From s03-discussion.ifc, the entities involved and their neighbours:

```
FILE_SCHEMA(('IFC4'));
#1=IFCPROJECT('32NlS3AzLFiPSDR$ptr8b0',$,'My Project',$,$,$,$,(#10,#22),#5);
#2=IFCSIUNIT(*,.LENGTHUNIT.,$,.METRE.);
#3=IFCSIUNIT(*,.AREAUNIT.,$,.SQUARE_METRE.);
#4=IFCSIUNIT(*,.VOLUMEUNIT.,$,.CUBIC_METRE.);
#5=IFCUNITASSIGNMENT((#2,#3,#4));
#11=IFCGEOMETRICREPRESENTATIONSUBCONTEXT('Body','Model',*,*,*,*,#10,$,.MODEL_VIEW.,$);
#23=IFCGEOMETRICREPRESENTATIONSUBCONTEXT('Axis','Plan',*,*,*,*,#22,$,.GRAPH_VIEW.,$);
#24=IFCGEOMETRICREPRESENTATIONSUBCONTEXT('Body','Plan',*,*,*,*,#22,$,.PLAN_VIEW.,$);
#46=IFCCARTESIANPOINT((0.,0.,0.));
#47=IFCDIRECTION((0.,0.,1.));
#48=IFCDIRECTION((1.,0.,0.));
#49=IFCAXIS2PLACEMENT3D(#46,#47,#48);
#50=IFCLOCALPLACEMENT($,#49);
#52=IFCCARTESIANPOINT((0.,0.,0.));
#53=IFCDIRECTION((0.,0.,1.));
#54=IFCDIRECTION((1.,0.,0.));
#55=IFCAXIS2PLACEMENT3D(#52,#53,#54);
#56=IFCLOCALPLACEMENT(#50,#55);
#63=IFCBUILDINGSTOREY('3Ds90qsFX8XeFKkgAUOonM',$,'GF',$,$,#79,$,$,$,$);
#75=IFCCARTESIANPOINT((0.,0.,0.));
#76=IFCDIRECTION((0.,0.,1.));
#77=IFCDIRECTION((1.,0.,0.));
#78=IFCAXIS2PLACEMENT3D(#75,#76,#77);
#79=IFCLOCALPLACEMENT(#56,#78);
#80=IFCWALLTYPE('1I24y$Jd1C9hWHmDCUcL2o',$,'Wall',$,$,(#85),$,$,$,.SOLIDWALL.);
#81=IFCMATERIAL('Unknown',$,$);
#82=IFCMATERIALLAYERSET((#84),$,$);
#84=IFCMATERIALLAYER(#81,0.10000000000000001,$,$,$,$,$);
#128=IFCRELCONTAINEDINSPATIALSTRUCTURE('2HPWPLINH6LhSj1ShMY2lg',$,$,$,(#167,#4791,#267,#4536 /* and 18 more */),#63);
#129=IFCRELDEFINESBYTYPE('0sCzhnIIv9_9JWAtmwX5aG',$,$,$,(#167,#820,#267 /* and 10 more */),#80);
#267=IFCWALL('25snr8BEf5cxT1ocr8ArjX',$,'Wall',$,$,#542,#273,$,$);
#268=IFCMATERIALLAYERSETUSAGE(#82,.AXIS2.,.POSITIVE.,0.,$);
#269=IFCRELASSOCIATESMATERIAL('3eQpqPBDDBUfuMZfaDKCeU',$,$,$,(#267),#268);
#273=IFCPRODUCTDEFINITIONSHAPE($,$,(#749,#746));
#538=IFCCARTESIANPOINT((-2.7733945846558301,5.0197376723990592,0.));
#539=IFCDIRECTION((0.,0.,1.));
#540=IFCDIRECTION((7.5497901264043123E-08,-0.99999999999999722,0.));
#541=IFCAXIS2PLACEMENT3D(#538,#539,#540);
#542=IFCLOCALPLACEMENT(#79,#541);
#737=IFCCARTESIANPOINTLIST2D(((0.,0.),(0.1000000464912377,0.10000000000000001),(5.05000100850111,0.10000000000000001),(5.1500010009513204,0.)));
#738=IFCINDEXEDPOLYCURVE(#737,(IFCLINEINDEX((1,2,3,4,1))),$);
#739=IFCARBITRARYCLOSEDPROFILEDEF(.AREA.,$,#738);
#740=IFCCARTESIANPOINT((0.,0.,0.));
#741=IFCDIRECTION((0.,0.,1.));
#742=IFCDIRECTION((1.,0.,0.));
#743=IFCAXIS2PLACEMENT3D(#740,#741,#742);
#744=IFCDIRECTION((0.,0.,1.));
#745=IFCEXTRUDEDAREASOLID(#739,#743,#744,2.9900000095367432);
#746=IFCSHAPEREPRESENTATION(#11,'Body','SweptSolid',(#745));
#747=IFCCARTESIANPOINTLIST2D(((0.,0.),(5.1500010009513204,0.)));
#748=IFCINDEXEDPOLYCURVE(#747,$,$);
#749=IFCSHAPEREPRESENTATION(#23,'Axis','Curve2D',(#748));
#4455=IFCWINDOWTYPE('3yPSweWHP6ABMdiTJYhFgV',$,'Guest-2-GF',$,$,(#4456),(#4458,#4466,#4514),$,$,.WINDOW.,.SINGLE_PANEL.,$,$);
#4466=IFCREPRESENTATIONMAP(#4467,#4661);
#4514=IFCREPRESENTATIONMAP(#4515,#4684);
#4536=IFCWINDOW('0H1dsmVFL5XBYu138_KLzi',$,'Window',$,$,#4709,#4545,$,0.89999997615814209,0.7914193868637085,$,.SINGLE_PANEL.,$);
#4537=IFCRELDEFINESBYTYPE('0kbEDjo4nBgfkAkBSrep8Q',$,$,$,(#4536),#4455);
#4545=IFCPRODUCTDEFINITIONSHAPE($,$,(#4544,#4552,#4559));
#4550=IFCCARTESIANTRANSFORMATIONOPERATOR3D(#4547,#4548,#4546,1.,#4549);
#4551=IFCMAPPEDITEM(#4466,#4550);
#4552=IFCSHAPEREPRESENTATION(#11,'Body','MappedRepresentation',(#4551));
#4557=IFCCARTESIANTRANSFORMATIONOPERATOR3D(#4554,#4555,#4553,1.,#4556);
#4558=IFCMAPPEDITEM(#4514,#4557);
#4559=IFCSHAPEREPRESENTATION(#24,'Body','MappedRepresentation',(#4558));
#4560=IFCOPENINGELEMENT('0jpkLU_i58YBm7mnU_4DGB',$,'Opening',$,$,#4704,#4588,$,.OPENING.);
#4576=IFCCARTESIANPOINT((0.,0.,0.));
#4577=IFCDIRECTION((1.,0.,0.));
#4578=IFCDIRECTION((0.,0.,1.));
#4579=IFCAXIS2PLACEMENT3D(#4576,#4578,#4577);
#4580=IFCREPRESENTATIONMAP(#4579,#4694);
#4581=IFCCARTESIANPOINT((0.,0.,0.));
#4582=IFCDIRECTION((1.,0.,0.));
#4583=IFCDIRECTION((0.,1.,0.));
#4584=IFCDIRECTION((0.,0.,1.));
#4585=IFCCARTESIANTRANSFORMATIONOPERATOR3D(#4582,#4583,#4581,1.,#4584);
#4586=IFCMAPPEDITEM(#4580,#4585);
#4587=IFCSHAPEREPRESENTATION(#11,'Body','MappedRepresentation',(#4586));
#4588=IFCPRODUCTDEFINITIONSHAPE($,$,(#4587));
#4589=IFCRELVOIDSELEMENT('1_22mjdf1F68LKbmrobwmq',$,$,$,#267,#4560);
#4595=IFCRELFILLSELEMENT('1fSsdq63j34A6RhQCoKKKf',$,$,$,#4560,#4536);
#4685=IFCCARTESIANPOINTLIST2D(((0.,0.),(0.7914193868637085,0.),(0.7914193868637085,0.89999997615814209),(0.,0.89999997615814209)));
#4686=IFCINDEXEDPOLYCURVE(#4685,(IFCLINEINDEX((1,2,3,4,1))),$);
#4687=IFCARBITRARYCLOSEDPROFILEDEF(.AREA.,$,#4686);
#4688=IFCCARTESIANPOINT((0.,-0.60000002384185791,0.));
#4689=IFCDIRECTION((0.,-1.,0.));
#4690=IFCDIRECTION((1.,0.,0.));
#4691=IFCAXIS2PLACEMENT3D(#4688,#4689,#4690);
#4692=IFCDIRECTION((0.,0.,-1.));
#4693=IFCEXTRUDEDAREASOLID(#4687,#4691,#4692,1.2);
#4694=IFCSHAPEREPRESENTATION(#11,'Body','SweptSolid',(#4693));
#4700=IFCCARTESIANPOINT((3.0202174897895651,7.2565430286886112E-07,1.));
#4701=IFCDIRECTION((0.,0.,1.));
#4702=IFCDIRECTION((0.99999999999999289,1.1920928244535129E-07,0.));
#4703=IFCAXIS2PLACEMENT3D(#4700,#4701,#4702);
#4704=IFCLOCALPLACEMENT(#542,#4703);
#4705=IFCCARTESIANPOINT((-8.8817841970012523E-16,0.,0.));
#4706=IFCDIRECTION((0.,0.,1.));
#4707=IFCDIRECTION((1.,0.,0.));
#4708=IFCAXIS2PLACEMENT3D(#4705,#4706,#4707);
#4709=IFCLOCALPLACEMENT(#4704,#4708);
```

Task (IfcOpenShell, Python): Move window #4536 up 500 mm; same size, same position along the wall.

```python
import numpy as np
import ifcopenshell
import ifcopenshell.api.geometry
import ifcopenshell.util.placement
import ifcopenshell.util.unit

model = ifcopenshell.open("s03-discussion.ifc")
unit_scale = ifcopenshell.util.unit.calculate_unit_scale(model)

window = model.by_guid("0H1dsmVFL5XBYu138_KLzi")
opening = window.FillsVoids[0].RelatingOpeningElement
dz = 0.5 / unit_scale

shift = np.array([0.0, 0.0, dz])
# The window is placed relative to its opening, so it follows when the opening moves.
matrix = ifcopenshell.util.placement.get_local_placement(opening.ObjectPlacement)
matrix[:3, 3] += shift
ifcopenshell.api.geometry.edit_object_placement(
    model, product=opening, matrix=matrix, is_si=False, should_transform_children=True
)

print(f"moved by {dz * unit_scale:+.3f} m")

model.write("s03-discussion_rev.ifc")
```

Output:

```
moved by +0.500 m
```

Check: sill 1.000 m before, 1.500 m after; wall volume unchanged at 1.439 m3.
